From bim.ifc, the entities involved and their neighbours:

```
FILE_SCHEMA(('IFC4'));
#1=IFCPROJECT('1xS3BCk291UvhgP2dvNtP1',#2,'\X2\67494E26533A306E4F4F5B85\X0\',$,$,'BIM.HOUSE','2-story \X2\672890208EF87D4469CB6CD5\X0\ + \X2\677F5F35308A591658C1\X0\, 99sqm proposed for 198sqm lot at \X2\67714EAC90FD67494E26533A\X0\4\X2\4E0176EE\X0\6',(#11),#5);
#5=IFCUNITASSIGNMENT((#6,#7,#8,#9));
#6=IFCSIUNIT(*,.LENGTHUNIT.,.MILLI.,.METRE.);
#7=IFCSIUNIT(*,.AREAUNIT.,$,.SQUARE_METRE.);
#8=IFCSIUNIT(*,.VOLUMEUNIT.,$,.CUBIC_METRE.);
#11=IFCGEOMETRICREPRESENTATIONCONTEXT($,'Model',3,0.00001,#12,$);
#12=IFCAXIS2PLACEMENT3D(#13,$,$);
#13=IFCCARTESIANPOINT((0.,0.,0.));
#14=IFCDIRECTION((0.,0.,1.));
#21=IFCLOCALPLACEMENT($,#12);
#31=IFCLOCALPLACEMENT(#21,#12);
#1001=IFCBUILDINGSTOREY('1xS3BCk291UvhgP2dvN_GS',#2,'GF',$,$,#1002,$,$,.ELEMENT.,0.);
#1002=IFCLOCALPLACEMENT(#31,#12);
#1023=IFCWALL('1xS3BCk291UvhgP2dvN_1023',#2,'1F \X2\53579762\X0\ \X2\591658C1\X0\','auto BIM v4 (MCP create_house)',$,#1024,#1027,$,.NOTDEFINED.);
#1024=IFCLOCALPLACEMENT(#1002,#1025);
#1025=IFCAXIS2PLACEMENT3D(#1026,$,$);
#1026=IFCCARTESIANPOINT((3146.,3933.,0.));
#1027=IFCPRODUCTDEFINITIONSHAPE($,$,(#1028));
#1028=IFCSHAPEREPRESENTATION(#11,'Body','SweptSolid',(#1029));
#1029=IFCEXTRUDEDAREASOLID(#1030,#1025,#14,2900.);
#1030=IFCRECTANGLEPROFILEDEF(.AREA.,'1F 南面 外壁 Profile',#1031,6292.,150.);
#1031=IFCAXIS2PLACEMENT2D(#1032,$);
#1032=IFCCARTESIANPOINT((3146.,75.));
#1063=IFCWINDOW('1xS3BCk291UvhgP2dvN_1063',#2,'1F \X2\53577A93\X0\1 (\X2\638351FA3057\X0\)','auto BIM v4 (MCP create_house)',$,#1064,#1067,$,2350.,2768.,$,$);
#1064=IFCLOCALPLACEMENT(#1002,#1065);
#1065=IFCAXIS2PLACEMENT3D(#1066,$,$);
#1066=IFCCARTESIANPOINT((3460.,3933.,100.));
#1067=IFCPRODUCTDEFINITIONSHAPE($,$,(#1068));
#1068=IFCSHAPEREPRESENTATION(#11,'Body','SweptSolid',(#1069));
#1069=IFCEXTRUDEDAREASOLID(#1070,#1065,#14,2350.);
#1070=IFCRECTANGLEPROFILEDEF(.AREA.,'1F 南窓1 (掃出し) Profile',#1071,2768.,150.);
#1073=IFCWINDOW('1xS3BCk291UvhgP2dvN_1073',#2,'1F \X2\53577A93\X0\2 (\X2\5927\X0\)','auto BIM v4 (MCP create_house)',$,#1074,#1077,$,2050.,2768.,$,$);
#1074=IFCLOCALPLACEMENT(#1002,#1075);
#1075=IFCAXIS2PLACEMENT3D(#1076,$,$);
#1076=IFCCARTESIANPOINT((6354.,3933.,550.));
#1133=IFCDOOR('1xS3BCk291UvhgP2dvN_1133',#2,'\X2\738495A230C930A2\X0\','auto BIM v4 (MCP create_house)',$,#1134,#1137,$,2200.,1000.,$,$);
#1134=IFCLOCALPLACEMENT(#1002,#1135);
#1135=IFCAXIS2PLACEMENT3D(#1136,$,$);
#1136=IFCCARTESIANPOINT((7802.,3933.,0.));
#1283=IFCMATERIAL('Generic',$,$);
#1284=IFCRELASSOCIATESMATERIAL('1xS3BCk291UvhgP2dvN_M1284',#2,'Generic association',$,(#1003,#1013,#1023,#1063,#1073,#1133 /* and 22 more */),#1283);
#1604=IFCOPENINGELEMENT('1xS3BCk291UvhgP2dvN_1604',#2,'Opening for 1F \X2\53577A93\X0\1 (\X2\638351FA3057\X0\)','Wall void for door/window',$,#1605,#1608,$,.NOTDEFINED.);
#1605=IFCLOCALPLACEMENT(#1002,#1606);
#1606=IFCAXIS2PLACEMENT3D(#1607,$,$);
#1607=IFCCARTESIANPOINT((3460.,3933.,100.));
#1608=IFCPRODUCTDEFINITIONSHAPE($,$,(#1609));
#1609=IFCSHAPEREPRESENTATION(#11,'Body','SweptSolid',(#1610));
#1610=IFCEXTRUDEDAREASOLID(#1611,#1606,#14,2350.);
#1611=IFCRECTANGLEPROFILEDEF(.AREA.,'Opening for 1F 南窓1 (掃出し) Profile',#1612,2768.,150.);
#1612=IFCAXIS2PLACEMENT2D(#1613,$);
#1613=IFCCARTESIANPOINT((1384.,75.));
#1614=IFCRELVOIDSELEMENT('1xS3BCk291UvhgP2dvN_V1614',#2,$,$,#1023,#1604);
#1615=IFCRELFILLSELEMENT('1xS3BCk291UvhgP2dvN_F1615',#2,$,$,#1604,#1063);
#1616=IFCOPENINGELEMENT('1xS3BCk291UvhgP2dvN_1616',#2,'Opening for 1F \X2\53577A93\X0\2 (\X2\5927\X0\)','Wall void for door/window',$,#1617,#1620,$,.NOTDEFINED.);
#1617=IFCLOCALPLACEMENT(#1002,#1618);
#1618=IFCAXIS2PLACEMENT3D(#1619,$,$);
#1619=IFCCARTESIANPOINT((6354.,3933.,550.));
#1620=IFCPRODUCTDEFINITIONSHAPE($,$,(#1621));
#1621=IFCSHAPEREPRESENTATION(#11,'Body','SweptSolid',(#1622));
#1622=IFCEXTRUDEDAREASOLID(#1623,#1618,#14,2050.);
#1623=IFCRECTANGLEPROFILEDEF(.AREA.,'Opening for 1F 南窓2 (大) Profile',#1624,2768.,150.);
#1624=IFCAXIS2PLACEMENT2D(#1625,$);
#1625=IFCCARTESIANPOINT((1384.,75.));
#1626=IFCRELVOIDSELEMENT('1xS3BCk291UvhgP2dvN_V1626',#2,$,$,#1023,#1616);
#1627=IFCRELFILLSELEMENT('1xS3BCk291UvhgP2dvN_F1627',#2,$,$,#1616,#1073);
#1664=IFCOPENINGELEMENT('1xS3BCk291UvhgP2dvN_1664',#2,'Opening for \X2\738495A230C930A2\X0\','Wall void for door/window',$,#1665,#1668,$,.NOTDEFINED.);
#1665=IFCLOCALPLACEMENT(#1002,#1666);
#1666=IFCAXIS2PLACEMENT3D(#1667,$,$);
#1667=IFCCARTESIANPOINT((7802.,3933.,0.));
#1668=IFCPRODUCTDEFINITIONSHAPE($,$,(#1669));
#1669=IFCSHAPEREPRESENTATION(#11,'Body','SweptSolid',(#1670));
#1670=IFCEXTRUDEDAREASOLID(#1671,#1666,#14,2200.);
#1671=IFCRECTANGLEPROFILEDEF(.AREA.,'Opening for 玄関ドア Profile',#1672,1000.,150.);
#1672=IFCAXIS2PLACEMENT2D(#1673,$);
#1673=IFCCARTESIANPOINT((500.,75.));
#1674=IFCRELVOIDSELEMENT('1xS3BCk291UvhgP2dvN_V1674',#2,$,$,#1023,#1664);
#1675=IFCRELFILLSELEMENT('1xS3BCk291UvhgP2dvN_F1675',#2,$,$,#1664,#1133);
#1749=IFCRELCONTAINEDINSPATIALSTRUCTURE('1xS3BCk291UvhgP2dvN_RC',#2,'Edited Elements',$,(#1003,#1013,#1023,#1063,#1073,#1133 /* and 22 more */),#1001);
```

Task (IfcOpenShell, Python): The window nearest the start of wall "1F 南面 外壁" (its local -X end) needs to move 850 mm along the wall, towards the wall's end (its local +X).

```python
import ifcopenshell
import ifcopenshell.api.geometry
import ifcopenshell.util.placement
import ifcopenshell.util.unit

model = ifcopenshell.open("bim.ifc")
unit_scale = ifcopenshell.util.unit.calculate_unit_scale(model)

window = model.by_guid("1xS3BCk291UvhgP2dvN_1063")
opening = window.FillsVoids[0].RelatingOpeningElement
wall = opening.VoidsElements[0].RelatingBuildingElement

wall_matrix = ifcopenshell.util.placement.get_local_placement(wall.ObjectPlacement)
shift = wall_matrix[:3, 0] * 0.85 / unit_scale
before = ifcopenshell.util.placement.get_local_placement(window.ObjectPlacement)[:3, 3].copy()

# The window is not placed relative to its opening, so move both.
for product in (opening, window):
    matrix = ifcopenshell.util.placement.get_local_placement(product.ObjectPlacement)
    matrix[:3, 3] += shift
    ifcopenshell.api.geometry.edit_object_placement(model, product=product, matrix=matrix, is_si=False)

after = ifcopenshell.util.placement.get_local_placement(window.ObjectPlacement)[:3, 3]
print("window moved by", (after - before).round(3) + 0.0)

model.write("bim_rev.ifc")
```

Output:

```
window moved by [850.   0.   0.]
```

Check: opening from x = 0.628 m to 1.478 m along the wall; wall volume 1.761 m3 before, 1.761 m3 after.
